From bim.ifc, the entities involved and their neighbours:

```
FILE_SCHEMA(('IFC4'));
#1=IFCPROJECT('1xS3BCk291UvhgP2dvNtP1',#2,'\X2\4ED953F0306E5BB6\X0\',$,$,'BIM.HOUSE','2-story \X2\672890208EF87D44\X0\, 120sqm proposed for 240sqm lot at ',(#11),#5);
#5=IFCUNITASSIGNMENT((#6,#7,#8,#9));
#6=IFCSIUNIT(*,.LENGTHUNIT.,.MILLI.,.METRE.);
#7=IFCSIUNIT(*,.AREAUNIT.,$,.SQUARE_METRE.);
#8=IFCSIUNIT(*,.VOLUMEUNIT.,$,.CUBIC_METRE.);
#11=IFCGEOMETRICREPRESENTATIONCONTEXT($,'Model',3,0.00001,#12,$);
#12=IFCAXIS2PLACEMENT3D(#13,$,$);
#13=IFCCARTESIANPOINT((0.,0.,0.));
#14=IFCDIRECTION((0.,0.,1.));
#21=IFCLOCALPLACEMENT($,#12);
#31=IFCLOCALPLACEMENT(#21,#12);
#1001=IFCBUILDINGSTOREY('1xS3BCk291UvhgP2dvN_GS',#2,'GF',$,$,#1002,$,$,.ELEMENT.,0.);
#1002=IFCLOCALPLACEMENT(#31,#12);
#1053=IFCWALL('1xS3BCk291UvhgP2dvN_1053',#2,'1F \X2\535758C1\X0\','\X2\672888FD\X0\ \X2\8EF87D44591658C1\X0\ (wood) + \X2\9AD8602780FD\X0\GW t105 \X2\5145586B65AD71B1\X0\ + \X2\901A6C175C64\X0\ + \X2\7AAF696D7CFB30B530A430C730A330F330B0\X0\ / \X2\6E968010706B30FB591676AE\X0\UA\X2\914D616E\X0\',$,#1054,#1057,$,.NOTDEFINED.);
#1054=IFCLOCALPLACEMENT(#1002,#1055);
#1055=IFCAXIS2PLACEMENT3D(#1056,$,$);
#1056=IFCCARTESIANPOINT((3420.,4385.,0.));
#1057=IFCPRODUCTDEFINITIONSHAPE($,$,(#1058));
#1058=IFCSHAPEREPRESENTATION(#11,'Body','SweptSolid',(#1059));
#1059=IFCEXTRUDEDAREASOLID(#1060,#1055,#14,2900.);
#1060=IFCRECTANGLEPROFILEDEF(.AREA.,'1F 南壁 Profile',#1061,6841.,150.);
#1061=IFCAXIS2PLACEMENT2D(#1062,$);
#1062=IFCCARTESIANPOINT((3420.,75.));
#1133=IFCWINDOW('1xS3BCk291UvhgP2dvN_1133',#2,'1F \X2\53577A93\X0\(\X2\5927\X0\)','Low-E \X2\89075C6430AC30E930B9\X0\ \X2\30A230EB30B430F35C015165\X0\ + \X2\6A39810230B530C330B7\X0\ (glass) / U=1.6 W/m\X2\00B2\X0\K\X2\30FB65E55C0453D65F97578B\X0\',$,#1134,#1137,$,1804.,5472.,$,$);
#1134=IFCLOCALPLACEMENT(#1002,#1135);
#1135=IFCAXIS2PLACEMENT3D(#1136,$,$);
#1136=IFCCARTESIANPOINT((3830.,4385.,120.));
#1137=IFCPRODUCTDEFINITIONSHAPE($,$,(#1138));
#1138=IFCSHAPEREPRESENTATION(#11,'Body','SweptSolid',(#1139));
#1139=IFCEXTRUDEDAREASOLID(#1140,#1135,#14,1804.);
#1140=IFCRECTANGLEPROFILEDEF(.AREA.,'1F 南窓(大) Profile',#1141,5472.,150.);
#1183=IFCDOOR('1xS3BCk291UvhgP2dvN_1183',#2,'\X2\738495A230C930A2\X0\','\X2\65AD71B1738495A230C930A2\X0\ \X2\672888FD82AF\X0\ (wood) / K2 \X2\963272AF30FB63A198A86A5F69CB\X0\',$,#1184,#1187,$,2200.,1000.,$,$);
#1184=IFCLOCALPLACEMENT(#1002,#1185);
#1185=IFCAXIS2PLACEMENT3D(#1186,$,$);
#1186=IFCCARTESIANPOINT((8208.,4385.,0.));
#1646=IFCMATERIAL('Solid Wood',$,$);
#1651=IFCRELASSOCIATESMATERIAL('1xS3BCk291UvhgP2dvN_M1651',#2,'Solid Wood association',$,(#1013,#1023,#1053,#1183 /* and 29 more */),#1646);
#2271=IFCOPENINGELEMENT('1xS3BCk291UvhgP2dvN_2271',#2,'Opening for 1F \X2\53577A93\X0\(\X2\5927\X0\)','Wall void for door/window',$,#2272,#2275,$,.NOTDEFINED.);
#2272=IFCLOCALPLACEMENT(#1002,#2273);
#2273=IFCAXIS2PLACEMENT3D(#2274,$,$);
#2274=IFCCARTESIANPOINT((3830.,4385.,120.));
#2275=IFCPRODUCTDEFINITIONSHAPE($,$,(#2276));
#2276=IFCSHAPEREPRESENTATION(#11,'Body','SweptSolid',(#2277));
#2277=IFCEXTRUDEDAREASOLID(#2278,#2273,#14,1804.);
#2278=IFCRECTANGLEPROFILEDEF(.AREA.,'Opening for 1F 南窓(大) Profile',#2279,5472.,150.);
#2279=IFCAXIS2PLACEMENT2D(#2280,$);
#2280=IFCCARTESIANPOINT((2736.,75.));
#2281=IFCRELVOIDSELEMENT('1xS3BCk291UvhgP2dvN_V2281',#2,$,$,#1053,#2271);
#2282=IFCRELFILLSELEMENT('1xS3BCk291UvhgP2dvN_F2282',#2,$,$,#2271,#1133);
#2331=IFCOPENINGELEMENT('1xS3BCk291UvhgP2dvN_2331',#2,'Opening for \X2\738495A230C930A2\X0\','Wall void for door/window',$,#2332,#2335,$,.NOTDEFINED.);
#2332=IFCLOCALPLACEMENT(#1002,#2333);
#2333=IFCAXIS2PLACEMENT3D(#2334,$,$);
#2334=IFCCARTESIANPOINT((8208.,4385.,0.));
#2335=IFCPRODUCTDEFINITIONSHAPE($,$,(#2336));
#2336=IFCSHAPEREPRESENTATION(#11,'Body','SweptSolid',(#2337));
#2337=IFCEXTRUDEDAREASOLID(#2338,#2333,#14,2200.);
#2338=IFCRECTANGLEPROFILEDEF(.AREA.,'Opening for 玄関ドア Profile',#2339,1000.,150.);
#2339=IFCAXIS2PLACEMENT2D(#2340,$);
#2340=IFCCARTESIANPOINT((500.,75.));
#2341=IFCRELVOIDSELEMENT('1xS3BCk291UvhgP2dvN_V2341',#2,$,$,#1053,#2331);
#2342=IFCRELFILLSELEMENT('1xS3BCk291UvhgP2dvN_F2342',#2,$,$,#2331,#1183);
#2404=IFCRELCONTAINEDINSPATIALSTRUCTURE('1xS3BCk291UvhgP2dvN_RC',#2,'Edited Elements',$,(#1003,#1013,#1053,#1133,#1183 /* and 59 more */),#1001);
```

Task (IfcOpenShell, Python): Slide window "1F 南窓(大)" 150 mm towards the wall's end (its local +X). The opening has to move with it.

```python
import ifcopenshell
import ifcopenshell.api.geometry
import ifcopenshell.util.placement
import ifcopenshell.util.unit

model = ifcopenshell.open("bim.ifc")
unit_scale = ifcopenshell.util.unit.calculate_unit_scale(model)

window = model.by_id(1133)
opening = window.FillsVoids[0].RelatingOpeningElement
wall = opening.VoidsElements[0].RelatingBuildingElement

wall_matrix = ifcopenshell.util.placement.get_local_placement(wall.ObjectPlacement)
shift = wall_matrix[:3, 0] * 0.15 / unit_scale
before = ifcopenshell.util.placement.get_local_placement(window.ObjectPlacement)[:3, 3].copy()

# The window is not placed relative to its opening, so move both.
for product in (opening, window):
    matrix = ifcopenshell.util.placement.get_local_placement(product.ObjectPlacement)
    matrix[:3, 3] += shift
    ifcopenshell.api.geometry.edit_object_placement(model, product=product, matrix=matrix, is_si=False)

after = ifcopenshell.util.placement.get_local_placement(window.ObjectPlacement)[:3, 3]
print("window moved by", (after - before).round(3) + 0.0)

model.write("bim-out.ifc")
```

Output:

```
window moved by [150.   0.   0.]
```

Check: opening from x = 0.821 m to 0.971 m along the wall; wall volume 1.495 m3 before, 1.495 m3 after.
